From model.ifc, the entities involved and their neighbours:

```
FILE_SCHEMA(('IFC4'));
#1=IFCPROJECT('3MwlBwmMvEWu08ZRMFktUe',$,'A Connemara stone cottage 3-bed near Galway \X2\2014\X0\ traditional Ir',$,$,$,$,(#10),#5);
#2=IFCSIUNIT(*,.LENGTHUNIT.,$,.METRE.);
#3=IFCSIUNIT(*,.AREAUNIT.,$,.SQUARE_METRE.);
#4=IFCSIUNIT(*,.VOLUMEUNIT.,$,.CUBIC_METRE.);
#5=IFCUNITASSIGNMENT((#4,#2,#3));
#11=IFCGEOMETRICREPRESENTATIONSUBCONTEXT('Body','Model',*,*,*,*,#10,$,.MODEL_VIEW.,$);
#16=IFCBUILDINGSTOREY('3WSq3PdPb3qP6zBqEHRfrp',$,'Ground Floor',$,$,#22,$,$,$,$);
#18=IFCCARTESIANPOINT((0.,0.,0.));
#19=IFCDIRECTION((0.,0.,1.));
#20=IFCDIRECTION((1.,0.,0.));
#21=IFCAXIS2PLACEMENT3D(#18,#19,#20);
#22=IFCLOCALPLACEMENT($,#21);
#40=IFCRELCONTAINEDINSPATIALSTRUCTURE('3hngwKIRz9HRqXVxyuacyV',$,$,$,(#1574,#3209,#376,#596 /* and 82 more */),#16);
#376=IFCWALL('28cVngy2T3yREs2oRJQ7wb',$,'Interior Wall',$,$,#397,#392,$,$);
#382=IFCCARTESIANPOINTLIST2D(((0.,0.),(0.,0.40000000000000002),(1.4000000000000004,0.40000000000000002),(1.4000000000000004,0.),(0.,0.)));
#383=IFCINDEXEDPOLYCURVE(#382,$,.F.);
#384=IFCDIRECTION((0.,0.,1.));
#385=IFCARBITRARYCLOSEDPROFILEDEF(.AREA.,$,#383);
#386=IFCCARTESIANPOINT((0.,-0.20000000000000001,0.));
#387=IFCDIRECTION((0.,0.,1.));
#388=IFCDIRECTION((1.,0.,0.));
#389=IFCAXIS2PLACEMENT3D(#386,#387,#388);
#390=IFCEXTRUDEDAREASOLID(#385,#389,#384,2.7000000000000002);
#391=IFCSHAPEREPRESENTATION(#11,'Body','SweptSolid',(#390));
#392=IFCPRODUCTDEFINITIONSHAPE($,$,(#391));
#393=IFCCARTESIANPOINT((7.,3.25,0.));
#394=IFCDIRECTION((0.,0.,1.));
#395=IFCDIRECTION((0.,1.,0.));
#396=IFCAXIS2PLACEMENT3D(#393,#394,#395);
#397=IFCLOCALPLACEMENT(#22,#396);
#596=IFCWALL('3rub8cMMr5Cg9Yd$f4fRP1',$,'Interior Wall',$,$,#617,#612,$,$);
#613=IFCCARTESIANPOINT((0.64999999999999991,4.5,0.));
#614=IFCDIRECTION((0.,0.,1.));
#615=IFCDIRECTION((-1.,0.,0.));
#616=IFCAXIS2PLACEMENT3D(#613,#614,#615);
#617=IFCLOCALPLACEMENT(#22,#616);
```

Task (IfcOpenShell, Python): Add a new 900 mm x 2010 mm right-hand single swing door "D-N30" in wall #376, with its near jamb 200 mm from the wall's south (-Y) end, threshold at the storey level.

```python
import numpy as np
import ifcopenshell
import ifcopenshell.api.feature
import ifcopenshell.api.geometry
import ifcopenshell.api.root
import ifcopenshell.api.spatial
import ifcopenshell.geom
import ifcopenshell.util.element
import ifcopenshell.util.placement
import ifcopenshell.util.representation
import ifcopenshell.util.shape
import ifcopenshell.util.unit

model = ifcopenshell.open("model.ifc")
unit_scale = ifcopenshell.util.unit.calculate_unit_scale(model)
settings = ifcopenshell.geom.settings()


def volume(element):
    """Net volume in cubic metres, openings subtracted."""
    shape = ifcopenshell.geom.create_shape(settings, element)
    return ifcopenshell.util.shape.get_volume(shape.geometry)


wall = model.by_guid("28cVngy2T3yREs2oRJQ7wb")
storey = ifcopenshell.util.element.get_container(wall, ifc_class="IfcBuildingStorey")
context = ifcopenshell.util.representation.get_context(model, "Model", "Body", "MODEL_VIEW")
before = volume(wall)

width, height, from_end, sill = 0.9, 2.01, 0.2, 0.0  # metres

# The wall runs along its own X axis, and the end named is its -X end.
wall_shape = ifcopenshell.geom.create_shape(settings, wall)
x, y, z = ifcopenshell.util.shape.get_vertices(wall_shape.geometry).T
start = x.min() + from_end
face, thickness = float(y.min()), float(y.max() - y.min())
wall_matrix = ifcopenshell.util.placement.get_local_placement(wall.ObjectPlacement)
level = ifcopenshell.util.placement.get_local_placement(storey.ObjectPlacement)[2, 3]


def in_wall(x, y):
    """Placement at x, y metres in the wall's axes, at sill height."""
    matrix = wall_matrix.copy()
    matrix[:, 3] = wall_matrix @ np.array([x / unit_scale, y / unit_scale, 0.0, 1.0])
    matrix[2, 3] = level + sill / unit_scale
    return matrix


# Opening: a box that overshoots both wall faces by 50 mm.
opening = ifcopenshell.api.root.create_entity(model, ifc_class="IfcOpeningElement", predefined_type="OPENING")
box = ifcopenshell.api.geometry.add_wall_representation(
    model, context=context, length=width, height=height, thickness=thickness + 0.1
)
ifcopenshell.api.geometry.assign_representation(model, product=opening, representation=box)
ifcopenshell.api.geometry.edit_object_placement(model, product=opening, matrix=in_wall(start, face - 0.05), is_si=False)
ifcopenshell.api.feature.add_feature(model, feature=opening, element=wall)

door = ifcopenshell.api.root.create_entity(model, ifc_class="IfcDoor", name="D-N30", predefined_type="DOOR")
door.OverallWidth, door.OverallHeight = width / unit_scale, height / unit_scale
door.OperationType = "SINGLE_SWING_RIGHT"
body = ifcopenshell.api.geometry.add_door_representation(
    model,
    context=context,
    overall_width=door.OverallWidth,
    overall_height=door.OverallHeight,
    operation_type="SINGLE_SWING_RIGHT",
    lining_properties={"LiningDepth": thickness / unit_scale, "ThresholdDepth": thickness / unit_scale},
)
ifcopenshell.api.geometry.assign_representation(model, product=door, representation=body)
ifcopenshell.api.spatial.assign_container(model, products=[door], relating_structure=storey)
ifcopenshell.api.feature.add_filling(model, opening=opening, element=door)

# The lining spans the wall, so the door starts at the wall face.
ifcopenshell.api.geometry.edit_object_placement(model, product=door, matrix=in_wall(start, face), is_si=False)

after = volume(wall)

print(f"wall volume {before:.3f} -> {after:.3f} m3")

model.write("model_v2.ifc")
```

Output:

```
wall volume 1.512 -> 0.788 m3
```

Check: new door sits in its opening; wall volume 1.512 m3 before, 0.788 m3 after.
